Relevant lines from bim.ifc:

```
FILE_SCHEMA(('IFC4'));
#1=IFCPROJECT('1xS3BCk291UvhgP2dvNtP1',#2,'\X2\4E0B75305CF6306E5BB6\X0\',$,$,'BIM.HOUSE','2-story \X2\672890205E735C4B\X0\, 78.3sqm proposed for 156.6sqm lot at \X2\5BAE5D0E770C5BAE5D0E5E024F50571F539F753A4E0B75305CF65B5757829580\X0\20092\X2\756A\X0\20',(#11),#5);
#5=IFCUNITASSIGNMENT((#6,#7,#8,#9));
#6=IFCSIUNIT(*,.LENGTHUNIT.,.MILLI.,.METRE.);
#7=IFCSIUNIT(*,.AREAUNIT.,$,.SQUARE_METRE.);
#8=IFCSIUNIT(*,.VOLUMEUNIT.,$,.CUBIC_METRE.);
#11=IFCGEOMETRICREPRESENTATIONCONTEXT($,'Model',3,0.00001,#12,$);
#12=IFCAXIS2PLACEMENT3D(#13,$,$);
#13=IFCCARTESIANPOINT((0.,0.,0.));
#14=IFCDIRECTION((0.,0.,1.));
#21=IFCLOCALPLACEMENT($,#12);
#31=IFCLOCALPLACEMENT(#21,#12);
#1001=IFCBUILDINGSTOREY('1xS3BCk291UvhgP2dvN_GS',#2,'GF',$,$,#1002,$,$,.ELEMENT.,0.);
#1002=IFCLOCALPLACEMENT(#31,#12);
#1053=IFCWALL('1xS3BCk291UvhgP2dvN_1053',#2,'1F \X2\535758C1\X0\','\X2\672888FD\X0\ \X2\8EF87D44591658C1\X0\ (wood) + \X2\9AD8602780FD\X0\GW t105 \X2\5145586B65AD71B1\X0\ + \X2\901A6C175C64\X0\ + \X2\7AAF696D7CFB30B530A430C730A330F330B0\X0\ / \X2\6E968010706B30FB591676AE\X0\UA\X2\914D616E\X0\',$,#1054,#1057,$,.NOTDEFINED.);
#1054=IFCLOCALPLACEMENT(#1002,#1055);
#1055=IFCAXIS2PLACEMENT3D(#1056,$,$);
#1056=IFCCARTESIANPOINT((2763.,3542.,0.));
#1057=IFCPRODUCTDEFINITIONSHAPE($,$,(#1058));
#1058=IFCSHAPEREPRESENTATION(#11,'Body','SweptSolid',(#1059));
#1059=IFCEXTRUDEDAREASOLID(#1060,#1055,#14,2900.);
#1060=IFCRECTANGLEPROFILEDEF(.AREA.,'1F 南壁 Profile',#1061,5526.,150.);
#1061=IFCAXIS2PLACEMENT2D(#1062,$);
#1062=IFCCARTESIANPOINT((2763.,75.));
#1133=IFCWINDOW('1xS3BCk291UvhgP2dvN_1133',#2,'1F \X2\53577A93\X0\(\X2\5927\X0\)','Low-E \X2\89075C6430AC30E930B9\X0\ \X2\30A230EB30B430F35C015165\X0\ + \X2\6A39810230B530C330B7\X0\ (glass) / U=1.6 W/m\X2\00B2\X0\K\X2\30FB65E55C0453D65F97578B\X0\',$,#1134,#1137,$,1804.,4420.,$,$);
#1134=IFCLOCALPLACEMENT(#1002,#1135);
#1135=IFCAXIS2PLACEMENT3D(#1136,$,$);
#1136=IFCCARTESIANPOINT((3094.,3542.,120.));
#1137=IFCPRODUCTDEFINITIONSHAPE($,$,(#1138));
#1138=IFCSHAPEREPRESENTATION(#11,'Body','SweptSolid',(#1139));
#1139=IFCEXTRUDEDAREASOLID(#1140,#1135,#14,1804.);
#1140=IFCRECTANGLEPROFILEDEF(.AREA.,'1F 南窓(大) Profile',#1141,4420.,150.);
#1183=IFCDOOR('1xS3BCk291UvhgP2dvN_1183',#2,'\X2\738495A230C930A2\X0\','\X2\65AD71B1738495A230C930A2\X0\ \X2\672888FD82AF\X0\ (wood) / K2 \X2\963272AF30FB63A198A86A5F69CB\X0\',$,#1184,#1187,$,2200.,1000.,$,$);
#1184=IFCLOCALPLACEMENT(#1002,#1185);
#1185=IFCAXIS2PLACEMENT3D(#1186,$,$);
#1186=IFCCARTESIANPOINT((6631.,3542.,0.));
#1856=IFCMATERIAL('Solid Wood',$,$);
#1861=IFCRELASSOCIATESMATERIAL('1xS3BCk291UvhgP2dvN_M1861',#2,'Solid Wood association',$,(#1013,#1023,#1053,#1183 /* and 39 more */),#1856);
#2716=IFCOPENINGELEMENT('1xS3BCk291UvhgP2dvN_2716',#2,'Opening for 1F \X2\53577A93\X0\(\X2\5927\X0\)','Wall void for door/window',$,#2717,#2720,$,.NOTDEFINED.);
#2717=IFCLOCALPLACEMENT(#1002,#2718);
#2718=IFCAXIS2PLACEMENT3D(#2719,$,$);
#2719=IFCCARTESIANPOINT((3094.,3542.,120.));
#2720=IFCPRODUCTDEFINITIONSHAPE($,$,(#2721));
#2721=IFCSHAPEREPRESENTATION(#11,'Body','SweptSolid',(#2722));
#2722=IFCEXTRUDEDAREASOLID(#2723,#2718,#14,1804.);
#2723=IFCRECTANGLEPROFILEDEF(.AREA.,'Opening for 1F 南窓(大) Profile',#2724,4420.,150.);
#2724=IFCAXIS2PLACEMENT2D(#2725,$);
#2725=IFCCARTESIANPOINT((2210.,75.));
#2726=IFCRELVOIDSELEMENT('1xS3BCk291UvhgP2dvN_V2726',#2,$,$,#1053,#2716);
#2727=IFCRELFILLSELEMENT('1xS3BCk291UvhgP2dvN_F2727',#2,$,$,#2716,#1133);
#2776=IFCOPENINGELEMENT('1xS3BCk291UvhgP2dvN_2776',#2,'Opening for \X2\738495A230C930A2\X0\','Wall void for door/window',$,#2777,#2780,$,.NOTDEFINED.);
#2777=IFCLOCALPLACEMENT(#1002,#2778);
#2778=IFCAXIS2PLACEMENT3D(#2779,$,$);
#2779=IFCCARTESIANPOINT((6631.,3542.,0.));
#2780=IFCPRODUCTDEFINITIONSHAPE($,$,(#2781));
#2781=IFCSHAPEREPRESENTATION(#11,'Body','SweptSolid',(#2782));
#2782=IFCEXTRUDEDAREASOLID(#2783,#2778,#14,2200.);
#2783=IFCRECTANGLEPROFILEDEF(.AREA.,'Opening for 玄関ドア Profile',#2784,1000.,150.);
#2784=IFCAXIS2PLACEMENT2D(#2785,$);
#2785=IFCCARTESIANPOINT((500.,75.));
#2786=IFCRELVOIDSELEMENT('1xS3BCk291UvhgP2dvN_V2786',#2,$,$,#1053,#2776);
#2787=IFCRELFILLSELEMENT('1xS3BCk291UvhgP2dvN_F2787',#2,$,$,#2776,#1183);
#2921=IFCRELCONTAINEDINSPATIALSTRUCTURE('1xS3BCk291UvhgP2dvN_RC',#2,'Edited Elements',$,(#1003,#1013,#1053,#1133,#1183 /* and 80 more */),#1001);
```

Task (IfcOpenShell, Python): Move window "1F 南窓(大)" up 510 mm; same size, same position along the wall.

```python
import numpy as np
import ifcopenshell
import ifcopenshell.api.geometry
import ifcopenshell.util.placement
import ifcopenshell.util.unit

model = ifcopenshell.open("bim.ifc")
unit_scale = ifcopenshell.util.unit.calculate_unit_scale(model)

window = model.by_guid("1xS3BCk291UvhgP2dvN_1133")
opening = window.FillsVoids[0].RelatingOpeningElement
dz = 0.51 / unit_scale

shift = np.array([0.0, 0.0, dz])
# The window is not placed relative to its opening, so move both.
for product in (opening, window):
    matrix = ifcopenshell.util.placement.get_local_placement(product.ObjectPlacement)
    matrix[:3, 3] += shift
    ifcopenshell.api.geometry.edit_object_placement(model, product=product, matrix=matrix, is_si=False)

print(f"moved by {dz * unit_scale:+.3f} m")

model.write("bim_edited.ifc")
```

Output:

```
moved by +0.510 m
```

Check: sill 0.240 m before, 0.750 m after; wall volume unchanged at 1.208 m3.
